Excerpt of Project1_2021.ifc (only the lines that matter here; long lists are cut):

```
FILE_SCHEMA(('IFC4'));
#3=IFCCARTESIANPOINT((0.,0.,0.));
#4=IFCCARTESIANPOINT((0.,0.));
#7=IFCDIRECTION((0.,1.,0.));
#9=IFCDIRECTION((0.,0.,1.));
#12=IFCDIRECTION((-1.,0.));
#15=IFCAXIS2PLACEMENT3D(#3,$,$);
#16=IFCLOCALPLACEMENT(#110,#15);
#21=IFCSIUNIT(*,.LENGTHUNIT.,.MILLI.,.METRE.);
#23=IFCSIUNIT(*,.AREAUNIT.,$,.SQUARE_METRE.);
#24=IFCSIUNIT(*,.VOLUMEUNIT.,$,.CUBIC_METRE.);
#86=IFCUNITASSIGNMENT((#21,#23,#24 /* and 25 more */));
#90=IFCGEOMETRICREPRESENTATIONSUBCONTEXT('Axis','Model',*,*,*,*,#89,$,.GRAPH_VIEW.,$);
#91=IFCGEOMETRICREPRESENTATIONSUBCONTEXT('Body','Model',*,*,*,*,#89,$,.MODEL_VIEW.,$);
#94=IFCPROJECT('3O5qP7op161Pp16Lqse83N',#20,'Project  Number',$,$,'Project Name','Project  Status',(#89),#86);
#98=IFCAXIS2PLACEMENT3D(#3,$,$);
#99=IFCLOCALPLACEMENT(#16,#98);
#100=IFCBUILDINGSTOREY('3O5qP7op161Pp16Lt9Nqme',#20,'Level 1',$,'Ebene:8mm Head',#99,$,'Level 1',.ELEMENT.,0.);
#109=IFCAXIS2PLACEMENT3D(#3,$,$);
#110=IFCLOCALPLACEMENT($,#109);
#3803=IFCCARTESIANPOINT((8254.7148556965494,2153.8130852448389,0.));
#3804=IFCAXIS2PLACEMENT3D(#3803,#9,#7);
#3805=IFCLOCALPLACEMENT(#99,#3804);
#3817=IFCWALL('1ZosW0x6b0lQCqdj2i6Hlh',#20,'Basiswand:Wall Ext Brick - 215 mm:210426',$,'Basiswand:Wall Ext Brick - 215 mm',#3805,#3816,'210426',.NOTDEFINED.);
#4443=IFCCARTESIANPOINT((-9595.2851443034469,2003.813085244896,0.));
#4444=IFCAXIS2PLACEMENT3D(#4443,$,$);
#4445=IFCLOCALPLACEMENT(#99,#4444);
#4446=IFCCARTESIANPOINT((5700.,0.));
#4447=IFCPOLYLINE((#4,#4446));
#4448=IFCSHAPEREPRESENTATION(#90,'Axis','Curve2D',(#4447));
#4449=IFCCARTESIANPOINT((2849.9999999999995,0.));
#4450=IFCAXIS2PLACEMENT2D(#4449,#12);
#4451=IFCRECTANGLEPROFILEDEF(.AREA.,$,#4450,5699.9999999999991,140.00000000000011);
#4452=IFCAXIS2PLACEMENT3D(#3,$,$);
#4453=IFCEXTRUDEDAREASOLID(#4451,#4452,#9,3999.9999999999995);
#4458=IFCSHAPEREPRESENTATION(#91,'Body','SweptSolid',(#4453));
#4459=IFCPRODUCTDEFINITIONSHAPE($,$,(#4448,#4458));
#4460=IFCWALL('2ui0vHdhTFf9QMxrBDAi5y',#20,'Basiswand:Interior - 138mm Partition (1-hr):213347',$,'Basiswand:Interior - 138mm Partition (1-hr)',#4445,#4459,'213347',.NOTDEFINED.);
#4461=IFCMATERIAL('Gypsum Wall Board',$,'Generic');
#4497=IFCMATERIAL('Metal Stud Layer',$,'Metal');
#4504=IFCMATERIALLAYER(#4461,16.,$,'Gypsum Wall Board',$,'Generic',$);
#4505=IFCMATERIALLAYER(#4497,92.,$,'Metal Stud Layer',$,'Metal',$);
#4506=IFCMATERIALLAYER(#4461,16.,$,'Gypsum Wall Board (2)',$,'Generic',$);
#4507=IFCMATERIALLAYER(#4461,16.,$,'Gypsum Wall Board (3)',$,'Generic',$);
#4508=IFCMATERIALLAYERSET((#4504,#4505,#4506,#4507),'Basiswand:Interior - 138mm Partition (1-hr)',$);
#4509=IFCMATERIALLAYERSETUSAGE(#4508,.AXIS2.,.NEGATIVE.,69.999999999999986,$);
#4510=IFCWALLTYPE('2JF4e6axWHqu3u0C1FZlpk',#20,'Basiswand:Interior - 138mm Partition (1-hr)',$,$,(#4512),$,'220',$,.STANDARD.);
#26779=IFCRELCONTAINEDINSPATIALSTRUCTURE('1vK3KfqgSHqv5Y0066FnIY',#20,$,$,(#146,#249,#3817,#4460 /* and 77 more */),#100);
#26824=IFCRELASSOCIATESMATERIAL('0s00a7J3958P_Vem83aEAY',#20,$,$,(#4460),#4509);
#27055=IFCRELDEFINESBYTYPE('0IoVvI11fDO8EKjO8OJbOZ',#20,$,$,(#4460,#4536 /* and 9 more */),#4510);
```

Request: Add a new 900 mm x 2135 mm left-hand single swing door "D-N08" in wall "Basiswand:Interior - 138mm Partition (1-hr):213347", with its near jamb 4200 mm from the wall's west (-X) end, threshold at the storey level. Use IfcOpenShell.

```python
import numpy as np
import ifcopenshell
import ifcopenshell.api.feature
import ifcopenshell.api.geometry
import ifcopenshell.api.root
import ifcopenshell.api.spatial
import ifcopenshell.geom
import ifcopenshell.util.element
import ifcopenshell.util.placement
import ifcopenshell.util.representation
import ifcopenshell.util.shape
import ifcopenshell.util.unit

model = ifcopenshell.open("Project1_2021.ifc")
unit_scale = ifcopenshell.util.unit.calculate_unit_scale(model)
settings = ifcopenshell.geom.settings()


def volume(element):
    """Net volume in cubic metres, openings subtracted."""
    shape = ifcopenshell.geom.create_shape(settings, element)
    return ifcopenshell.util.shape.get_volume(shape.geometry)


wall = model.by_guid("2ui0vHdhTFf9QMxrBDAi5y")
storey = ifcopenshell.util.element.get_container(wall, ifc_class="IfcBuildingStorey")
context = ifcopenshell.util.representation.get_context(model, "Model", "Body", "MODEL_VIEW")
before = volume(wall)

width, height, from_end, sill = 0.9, 2.135, 4.2, 0.0  # metres

# The wall runs along its own X axis, and the end named is its -X end.
wall_shape = ifcopenshell.geom.create_shape(settings, wall)
x, y, z = ifcopenshell.util.shape.get_vertices(wall_shape.geometry).T
start = x.min() + from_end
face, thickness = float(y.min()), float(y.max() - y.min())
wall_matrix = ifcopenshell.util.placement.get_local_placement(wall.ObjectPlacement)
level = ifcopenshell.util.placement.get_local_placement(storey.ObjectPlacement)[2, 3]


def in_wall(x, y):
    """Placement at x, y metres in the wall's axes, at sill height."""
    matrix = wall_matrix.copy()
    matrix[:, 3] = wall_matrix @ np.array([x / unit_scale, y / unit_scale, 0.0, 1.0])
    matrix[2, 3] = level + sill / unit_scale
    return matrix


# Opening: a box that overshoots both wall faces by 50 mm.
opening = ifcopenshell.api.root.create_entity(model, ifc_class="IfcOpeningElement", predefined_type="OPENING")
box = ifcopenshell.api.geometry.add_wall_representation(
    model, context=context, length=width, height=height, thickness=thickness + 0.1
)
ifcopenshell.api.geometry.assign_representation(model, product=opening, representation=box)
ifcopenshell.api.geometry.edit_object_placement(model, product=opening, matrix=in_wall(start, face - 0.05), is_si=False)
ifcopenshell.api.feature.add_feature(model, feature=opening, element=wall)

door = ifcopenshell.api.root.create_entity(model, ifc_class="IfcDoor", name="D-N08", predefined_type="DOOR")
door.OverallWidth, door.OverallHeight = width / unit_scale, height / unit_scale
door.OperationType = "SINGLE_SWING_LEFT"
body = ifcopenshell.api.geometry.add_door_representation(
    model,
    context=context,
    overall_width=door.OverallWidth,
    overall_height=door.OverallHeight,
    operation_type="SINGLE_SWING_LEFT",
    lining_properties={"LiningDepth": thickness / unit_scale, "ThresholdDepth": thickness / unit_scale},
)
ifcopenshell.api.geometry.assign_representation(model, product=door, representation=body)
ifcopenshell.api.spatial.assign_container(model, products=[door], relating_structure=storey)
ifcopenshell.api.feature.add_filling(model, opening=opening, element=door)

# The lining spans the wall, so the door starts at the wall face.
ifcopenshell.api.geometry.edit_object_placement(model, product=door, matrix=in_wall(start, face), is_si=False)

after = volume(wall)

print(f"wall volume {before:.3f} -> {after:.3f} m3")

model.write("Project1_2021_v2.ifc")
```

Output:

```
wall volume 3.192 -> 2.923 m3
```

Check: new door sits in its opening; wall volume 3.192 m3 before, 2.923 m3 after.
